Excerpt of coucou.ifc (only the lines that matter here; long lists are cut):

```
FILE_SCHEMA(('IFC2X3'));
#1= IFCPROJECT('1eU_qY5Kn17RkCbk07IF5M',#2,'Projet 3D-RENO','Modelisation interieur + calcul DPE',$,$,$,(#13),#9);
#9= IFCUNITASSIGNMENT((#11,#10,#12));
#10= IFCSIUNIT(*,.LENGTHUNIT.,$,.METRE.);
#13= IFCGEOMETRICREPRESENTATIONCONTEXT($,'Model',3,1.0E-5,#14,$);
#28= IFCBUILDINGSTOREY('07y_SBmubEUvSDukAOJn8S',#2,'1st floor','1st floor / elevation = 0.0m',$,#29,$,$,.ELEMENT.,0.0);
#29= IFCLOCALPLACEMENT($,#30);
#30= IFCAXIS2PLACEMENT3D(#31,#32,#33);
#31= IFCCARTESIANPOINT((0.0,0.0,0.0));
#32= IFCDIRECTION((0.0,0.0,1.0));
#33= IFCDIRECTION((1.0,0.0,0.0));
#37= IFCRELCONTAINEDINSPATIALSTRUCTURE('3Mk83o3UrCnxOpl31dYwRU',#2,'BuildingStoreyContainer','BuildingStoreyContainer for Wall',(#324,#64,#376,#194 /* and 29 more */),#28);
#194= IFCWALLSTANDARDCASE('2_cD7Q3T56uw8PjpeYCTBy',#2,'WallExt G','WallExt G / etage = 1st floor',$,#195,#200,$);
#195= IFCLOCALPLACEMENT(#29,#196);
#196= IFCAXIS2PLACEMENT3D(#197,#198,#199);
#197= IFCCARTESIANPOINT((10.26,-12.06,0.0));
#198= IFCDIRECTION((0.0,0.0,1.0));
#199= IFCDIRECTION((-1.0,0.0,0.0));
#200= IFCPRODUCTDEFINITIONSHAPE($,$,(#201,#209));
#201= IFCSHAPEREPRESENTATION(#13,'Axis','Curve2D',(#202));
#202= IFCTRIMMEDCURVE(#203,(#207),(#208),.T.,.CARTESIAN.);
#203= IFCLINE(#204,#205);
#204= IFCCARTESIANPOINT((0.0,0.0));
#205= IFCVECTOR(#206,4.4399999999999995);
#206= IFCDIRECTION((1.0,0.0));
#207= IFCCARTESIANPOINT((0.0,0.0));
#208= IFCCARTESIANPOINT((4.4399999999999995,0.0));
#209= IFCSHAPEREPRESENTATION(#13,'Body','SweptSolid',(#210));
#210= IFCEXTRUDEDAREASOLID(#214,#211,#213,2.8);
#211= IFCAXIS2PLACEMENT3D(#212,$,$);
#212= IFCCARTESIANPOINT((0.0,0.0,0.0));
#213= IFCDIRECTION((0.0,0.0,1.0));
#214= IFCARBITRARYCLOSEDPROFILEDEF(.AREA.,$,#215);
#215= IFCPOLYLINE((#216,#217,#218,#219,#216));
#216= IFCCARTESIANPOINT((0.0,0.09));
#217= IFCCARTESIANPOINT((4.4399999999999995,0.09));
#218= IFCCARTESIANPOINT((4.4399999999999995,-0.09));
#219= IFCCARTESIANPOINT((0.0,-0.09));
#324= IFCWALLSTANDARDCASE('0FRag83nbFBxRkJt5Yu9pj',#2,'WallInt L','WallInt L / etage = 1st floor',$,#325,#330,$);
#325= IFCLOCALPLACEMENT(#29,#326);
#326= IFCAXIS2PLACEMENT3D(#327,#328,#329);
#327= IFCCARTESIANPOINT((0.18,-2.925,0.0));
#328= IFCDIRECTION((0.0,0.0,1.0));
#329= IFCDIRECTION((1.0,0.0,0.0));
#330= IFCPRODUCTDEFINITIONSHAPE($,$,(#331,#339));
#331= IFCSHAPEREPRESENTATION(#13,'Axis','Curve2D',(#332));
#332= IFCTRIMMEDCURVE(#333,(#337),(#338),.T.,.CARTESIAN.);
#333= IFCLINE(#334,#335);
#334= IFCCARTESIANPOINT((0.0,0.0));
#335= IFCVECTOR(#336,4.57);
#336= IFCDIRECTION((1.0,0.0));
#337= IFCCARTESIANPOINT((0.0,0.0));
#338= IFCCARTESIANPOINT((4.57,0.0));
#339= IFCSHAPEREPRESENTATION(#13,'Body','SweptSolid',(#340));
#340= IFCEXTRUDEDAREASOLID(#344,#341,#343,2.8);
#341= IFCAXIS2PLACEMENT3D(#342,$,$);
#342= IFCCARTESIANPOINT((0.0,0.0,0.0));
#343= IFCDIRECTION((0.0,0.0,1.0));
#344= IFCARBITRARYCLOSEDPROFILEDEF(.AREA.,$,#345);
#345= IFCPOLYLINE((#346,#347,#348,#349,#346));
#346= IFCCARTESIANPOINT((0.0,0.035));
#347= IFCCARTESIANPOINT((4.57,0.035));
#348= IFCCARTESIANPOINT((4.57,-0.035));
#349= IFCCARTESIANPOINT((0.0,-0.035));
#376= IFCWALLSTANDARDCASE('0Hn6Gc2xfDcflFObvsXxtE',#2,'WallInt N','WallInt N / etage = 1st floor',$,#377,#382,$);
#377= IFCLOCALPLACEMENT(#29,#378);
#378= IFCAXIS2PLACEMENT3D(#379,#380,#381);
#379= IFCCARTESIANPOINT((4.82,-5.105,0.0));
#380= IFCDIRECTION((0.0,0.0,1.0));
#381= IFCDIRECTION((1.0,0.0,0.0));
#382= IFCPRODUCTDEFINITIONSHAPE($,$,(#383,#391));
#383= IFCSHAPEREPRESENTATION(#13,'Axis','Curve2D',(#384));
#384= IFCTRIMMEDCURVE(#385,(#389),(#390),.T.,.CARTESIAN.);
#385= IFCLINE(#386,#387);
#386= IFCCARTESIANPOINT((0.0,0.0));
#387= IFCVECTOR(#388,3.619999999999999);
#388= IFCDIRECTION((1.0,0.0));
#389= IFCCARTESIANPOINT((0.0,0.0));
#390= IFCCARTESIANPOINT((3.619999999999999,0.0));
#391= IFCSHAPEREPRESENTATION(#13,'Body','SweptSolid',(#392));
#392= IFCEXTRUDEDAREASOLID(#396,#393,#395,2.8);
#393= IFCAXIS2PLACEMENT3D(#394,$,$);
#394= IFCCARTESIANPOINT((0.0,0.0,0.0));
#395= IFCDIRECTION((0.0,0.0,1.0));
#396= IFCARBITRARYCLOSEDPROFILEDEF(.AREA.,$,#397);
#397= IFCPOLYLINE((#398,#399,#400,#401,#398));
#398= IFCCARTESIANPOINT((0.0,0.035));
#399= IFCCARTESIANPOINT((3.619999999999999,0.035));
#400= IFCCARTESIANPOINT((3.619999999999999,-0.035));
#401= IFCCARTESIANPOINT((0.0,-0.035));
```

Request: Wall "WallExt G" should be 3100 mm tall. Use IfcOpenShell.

```python
import ifcopenshell
import ifcopenshell.geom
import ifcopenshell.util.shape
import ifcopenshell.util.unit

model = ifcopenshell.open("coucou.ifc")
unit_scale = ifcopenshell.util.unit.calculate_unit_scale(model)
settings = ifcopenshell.geom.settings()


def volume(element):
    """Net volume in cubic metres, openings subtracted."""
    shape = ifcopenshell.geom.create_shape(settings, element)
    return ifcopenshell.util.shape.get_volume(shape.geometry)


wall = model.by_guid("2_cD7Q3T56uw8PjpeYCTBy")
before = volume(wall)

body = next(r for r in wall.Representation.Representations if r.RepresentationIdentifier == "Body")
solid = body.Items[0]
old_height = solid.Depth
solid.Depth = 3.1 / unit_scale
after = volume(wall)

print(f"height {old_height:g} -> {solid.Depth:g}, volume {before:.3f} -> {after:.3f} m3")

model.write("coucou-out.ifc")
```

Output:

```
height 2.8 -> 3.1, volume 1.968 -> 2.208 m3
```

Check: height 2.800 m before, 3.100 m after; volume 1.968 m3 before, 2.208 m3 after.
